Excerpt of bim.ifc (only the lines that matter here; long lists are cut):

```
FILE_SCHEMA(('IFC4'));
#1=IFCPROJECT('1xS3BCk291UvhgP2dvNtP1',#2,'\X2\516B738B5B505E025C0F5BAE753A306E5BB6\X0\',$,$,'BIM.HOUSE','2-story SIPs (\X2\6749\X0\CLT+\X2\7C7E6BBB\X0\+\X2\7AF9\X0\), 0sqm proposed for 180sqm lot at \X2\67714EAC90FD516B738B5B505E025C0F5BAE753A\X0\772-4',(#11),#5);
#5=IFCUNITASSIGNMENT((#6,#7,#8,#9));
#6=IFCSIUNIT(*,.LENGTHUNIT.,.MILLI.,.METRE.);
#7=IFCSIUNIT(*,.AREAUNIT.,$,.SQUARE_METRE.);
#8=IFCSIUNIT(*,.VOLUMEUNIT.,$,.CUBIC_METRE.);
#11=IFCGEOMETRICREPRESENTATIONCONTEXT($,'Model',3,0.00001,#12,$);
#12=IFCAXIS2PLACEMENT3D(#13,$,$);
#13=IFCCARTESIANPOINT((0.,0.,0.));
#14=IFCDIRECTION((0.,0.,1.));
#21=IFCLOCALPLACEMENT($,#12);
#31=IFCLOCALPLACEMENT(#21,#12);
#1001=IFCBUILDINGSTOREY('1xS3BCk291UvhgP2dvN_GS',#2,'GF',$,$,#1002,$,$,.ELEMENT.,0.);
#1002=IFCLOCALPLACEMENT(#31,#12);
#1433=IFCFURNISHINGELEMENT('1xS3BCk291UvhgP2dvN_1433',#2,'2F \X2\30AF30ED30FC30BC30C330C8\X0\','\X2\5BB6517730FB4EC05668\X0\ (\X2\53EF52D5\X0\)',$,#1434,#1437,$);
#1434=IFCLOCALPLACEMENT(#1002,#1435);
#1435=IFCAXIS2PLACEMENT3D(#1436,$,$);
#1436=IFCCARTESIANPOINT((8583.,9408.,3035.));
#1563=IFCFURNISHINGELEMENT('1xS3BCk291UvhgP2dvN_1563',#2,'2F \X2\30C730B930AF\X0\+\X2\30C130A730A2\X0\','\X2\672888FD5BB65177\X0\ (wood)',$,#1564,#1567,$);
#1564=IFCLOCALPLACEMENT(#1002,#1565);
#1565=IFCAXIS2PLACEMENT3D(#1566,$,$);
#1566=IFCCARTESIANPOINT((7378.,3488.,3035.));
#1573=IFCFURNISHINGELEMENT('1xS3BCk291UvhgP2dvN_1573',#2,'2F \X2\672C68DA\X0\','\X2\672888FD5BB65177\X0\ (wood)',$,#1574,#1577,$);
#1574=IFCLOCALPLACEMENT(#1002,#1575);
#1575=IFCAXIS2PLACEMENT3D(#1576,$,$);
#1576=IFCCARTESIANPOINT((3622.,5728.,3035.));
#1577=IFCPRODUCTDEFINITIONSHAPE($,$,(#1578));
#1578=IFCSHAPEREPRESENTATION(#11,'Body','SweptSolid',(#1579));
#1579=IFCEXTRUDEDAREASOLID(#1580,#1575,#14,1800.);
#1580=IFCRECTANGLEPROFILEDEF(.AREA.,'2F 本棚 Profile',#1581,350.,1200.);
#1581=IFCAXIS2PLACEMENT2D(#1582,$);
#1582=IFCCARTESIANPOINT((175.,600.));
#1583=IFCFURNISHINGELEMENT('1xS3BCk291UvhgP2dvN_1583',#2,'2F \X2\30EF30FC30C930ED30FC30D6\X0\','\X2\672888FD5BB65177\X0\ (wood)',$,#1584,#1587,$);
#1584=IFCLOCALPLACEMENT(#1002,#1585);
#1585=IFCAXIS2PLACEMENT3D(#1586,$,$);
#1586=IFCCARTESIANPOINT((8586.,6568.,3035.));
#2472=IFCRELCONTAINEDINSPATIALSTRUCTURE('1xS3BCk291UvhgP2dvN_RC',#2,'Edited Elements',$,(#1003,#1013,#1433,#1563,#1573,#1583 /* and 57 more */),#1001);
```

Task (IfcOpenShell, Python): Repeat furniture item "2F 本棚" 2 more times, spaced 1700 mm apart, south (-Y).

```python
import numpy as np
import ifcopenshell
import ifcopenshell.api.geometry
import ifcopenshell.api.root
import ifcopenshell.util.element
import ifcopenshell.util.placement

model = ifcopenshell.open("bim.ifc")


def reuse_history(source, copy):
    """copy_class also copies each property set's owner history, people and application; keep the originals."""
    for rel in copy.IsDefinedBy:
        if rel.is_a("IfcRelDefinesByProperties") and (history := rel.RelatingPropertyDefinition.OwnerHistory):
            rel.RelatingPropertyDefinition.OwnerHistory = source.OwnerHistory
            ifcopenshell.util.element.remove_deep2(model, history)


source = model.by_guid("1xS3BCk291UvhgP2dvN_1573")
base = ifcopenshell.util.placement.get_local_placement(source.ObjectPlacement)
step = np.array([0.0, -1.0, 0.0]) * 1700.0

for i in range(1, 3):
    copy = ifcopenshell.api.root.copy_class(model, product=source)
    copy.Representation = ifcopenshell.util.element.copy_deep(
        model, source.Representation, exclude=["IfcGeometricRepresentationContext", "IfcRepresentationMap"]
    )
    reuse_history(source, copy)
    matrix = base.copy()
    matrix[:3, 3] += i * step
    print("added at", matrix[:3, 3].round(3) + 0.0)
    ifcopenshell.api.geometry.edit_object_placement(model, product=copy, matrix=matrix, is_si=False)

model.write("bim_edited.ifc")
```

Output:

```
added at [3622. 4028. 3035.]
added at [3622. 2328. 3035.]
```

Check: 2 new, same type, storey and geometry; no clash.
